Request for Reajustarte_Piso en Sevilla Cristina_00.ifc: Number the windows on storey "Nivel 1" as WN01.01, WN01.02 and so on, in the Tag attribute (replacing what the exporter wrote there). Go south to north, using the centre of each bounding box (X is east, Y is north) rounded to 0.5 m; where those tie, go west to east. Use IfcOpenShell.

First a look at what the model holds.

```python
import ifcopenshell
import ifcopenshell.util.element
import ifcopenshell.util.placement

model = ifcopenshell.open("Reajustarte_Piso en Sevilla Cristina_00.ifc")
print(model.schema)
storey = next(s for s in model.by_type("IfcBuildingStorey") if s.Name == "Nivel 1")
windows = [e for e in ifcopenshell.util.element.get_decomposition(storey) if e.is_a("IfcWindow")]
for e in sorted(windows, key=lambda e: e.id()):
    origin = ifcopenshell.util.placement.get_local_placement(e.ObjectPlacement)[:3, 3]
    print(e.id(), e.Tag, e.Name, origin.round(2) + 0.0, sep=" | ")
```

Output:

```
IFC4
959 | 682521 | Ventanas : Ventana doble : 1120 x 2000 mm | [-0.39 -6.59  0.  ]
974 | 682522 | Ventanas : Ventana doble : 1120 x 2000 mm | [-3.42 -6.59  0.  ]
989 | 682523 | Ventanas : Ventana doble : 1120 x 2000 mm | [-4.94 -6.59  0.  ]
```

```python
import ifcopenshell
import ifcopenshell.geom
import ifcopenshell.util.element
import ifcopenshell.util.shape

model = ifcopenshell.open("Reajustarte_Piso en Sevilla Cristina_00.ifc")
settings = ifcopenshell.geom.settings()
settings.set("use-world-coords", True)


def centre(element):
    shape = ifcopenshell.geom.create_shape(settings, element)
    return ifcopenshell.util.shape.get_bbox_centroid(shape.geometry)


storey = next(s for s in model.by_type("IfcBuildingStorey") if s.Name == "Nivel 1")
windows = [e for e in ifcopenshell.util.element.get_decomposition(storey) if e.is_a("IfcWindow")]

# Insertion points can sit at a corner or the storey origin, so sort by the geometry (in metres).
centres = {e: centre(e) for e in windows}
windows.sort(key=lambda e: (round(centres[e][1] / 0.5), centres[e][0]))

for i, e in enumerate(windows, start=1):
    number = f"WN01.{i:02d}"
    e.Tag = number
    print(e.id(), number)

model.write("Reajustarte_Piso en Sevilla Cristina_00-out.ifc")
```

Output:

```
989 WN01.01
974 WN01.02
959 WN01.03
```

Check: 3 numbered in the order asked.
